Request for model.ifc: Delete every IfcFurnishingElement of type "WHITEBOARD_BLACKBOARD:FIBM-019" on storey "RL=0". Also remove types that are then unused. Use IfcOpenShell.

First a look at what the model holds.

```python
import ifcopenshell
import ifcopenshell.util.element

model = ifcopenshell.open("model.ifc")
print(model.schema)
storey = next(s for s in model.by_type("IfcBuildingStorey") if s.Name == "RL=0")
furniture = [e for e in ifcopenshell.util.element.get_decomposition(storey) if e.is_a("IfcFurnishingElement")]
seen = {}
for e in furniture:
    element_type = ifcopenshell.util.element.get_type(e)
    name = element_type.Name if element_type not in (None, e) else None
    seen[name] = seen.get(name, 0) + 1
for name, count in sorted(seen.items(), key=str):
    print(count, "x", name)
```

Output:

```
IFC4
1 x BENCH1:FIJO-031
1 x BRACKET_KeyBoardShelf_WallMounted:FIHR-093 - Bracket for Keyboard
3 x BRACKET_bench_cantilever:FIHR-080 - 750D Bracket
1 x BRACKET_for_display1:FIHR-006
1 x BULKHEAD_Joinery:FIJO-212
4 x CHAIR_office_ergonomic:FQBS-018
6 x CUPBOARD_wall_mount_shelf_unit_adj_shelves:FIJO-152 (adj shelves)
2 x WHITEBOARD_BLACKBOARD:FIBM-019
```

```python
import ifcopenshell
import ifcopenshell.api.root
import ifcopenshell.util.element

model = ifcopenshell.open("model.ifc")

storey = next(s for s in model.by_type("IfcBuildingStorey") if s.Name == "RL=0")
furniture = [e for e in ifcopenshell.util.element.get_decomposition(storey) if e.is_a("IfcFurnishingElement")]
targets = [e for e in furniture if (t := ifcopenshell.util.element.get_type(e)) not in (None, e) and t.Name == "WHITEBOARD_BLACKBOARD:FIBM-019"]
types = {ifcopenshell.util.element.get_type(e) for e in targets} - {None, *targets}

for e in targets:
    ifcopenshell.api.root.remove_product(model, product=e)
print(len(targets), "removed")

unused = [t for t in types if not ifcopenshell.util.element.get_types(t)]
for t in unused:
    ifcopenshell.api.root.remove_product(model, product=t)
print(len(unused), "unused types removed")

model.write("model-out.ifc")
```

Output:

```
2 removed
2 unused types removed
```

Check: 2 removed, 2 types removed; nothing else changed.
